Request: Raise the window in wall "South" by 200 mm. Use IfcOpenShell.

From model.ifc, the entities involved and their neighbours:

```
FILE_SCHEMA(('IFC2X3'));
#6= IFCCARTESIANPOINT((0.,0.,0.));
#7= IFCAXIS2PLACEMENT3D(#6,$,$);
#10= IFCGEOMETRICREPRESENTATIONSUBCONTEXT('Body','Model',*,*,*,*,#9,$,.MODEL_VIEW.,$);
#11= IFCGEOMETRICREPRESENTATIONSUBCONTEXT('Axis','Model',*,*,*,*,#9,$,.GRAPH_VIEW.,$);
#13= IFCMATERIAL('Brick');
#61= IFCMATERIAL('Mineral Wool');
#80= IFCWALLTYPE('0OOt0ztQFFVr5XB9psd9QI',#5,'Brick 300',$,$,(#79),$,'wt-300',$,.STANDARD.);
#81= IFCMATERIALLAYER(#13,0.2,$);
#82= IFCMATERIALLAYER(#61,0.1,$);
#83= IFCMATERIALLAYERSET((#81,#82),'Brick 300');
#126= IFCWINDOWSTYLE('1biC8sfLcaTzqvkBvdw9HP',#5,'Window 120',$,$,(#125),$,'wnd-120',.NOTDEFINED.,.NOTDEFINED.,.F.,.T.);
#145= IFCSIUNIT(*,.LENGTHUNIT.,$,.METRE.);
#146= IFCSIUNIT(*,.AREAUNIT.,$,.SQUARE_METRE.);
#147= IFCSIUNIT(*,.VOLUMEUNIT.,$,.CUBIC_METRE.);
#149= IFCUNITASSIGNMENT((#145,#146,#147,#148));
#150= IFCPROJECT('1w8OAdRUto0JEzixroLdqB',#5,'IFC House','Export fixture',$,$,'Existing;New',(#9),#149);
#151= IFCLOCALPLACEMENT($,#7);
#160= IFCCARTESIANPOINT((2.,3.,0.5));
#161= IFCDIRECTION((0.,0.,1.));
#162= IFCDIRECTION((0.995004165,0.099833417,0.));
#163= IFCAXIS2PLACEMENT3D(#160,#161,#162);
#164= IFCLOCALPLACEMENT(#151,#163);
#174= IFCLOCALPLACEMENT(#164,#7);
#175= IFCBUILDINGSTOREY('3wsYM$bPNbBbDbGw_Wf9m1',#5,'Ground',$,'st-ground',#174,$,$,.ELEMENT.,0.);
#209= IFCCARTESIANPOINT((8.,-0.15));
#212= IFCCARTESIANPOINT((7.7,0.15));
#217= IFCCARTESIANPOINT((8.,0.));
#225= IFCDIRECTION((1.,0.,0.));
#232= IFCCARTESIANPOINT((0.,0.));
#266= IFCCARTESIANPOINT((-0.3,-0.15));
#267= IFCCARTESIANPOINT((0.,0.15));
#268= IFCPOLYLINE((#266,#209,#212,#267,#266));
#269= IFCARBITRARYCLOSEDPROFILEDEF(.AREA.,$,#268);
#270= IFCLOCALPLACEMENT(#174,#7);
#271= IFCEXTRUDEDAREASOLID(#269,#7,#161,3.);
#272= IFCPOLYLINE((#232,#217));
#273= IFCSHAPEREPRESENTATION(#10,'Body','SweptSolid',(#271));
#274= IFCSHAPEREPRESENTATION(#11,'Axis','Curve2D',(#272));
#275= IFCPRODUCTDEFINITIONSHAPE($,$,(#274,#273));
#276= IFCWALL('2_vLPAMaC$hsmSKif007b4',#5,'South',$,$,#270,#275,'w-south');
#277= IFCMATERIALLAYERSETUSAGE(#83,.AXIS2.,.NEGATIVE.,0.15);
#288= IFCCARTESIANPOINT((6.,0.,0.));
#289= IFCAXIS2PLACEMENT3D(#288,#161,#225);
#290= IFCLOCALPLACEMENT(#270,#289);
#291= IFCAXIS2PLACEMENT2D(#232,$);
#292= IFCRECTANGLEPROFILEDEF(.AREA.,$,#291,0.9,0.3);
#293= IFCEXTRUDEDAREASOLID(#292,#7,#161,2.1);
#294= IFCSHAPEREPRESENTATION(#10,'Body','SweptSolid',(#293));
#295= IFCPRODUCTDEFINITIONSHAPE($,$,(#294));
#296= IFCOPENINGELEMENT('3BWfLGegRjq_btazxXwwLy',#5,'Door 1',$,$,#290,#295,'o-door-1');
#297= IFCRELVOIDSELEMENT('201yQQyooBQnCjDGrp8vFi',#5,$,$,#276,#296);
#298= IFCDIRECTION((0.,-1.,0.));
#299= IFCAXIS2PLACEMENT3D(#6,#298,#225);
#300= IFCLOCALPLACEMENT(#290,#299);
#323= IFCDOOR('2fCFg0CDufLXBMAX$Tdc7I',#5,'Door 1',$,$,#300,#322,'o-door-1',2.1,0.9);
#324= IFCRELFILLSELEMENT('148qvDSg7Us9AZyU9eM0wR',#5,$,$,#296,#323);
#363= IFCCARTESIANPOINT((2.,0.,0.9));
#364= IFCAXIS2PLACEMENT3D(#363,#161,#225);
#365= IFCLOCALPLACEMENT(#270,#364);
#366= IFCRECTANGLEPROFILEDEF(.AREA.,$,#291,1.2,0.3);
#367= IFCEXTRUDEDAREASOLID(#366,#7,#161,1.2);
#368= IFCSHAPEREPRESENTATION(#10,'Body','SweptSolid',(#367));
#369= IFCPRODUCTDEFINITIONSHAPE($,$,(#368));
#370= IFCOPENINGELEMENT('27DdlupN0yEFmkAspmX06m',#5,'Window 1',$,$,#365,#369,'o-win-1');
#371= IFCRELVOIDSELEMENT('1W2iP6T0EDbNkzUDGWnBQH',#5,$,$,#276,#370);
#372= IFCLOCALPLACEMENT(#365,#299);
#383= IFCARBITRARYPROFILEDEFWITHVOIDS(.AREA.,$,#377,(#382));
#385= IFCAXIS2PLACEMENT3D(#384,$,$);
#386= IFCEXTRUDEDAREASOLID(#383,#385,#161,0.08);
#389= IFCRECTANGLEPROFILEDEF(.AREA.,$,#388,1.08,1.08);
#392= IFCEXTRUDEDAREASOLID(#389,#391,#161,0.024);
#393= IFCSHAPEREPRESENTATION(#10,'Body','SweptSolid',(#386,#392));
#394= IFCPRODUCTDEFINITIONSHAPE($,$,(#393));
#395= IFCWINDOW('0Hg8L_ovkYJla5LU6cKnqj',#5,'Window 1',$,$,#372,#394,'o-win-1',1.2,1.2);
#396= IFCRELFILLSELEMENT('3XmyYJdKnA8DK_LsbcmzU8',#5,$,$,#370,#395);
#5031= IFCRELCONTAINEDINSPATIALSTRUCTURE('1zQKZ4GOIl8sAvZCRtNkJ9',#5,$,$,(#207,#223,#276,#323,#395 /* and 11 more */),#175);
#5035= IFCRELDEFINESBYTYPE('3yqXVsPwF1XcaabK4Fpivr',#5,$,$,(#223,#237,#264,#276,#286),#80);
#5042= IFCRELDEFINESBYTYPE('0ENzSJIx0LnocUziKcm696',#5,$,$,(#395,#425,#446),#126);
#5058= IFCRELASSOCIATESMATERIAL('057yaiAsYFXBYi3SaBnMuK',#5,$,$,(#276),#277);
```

```python
import numpy as np
import ifcopenshell
import ifcopenshell.api.geometry
import ifcopenshell.util.placement
import ifcopenshell.util.unit

model = ifcopenshell.open("model.ifc")
unit_scale = ifcopenshell.util.unit.calculate_unit_scale(model)

window = model.by_id(395)
opening = window.FillsVoids[0].RelatingOpeningElement
dz = 0.2

shift = np.array([0.0, 0.0, dz])
# The window is placed relative to its opening, so it follows when the opening moves.
matrix = ifcopenshell.util.placement.get_local_placement(opening.ObjectPlacement)
matrix[:3, 3] += shift
ifcopenshell.api.geometry.edit_object_placement(
    model, product=opening, matrix=matrix, is_si=False, should_transform_children=True
)

print(f"moved by {dz * unit_scale:+.3f} m")

model.write("model_edited.ifc")
```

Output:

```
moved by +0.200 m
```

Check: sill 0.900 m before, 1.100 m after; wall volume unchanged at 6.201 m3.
